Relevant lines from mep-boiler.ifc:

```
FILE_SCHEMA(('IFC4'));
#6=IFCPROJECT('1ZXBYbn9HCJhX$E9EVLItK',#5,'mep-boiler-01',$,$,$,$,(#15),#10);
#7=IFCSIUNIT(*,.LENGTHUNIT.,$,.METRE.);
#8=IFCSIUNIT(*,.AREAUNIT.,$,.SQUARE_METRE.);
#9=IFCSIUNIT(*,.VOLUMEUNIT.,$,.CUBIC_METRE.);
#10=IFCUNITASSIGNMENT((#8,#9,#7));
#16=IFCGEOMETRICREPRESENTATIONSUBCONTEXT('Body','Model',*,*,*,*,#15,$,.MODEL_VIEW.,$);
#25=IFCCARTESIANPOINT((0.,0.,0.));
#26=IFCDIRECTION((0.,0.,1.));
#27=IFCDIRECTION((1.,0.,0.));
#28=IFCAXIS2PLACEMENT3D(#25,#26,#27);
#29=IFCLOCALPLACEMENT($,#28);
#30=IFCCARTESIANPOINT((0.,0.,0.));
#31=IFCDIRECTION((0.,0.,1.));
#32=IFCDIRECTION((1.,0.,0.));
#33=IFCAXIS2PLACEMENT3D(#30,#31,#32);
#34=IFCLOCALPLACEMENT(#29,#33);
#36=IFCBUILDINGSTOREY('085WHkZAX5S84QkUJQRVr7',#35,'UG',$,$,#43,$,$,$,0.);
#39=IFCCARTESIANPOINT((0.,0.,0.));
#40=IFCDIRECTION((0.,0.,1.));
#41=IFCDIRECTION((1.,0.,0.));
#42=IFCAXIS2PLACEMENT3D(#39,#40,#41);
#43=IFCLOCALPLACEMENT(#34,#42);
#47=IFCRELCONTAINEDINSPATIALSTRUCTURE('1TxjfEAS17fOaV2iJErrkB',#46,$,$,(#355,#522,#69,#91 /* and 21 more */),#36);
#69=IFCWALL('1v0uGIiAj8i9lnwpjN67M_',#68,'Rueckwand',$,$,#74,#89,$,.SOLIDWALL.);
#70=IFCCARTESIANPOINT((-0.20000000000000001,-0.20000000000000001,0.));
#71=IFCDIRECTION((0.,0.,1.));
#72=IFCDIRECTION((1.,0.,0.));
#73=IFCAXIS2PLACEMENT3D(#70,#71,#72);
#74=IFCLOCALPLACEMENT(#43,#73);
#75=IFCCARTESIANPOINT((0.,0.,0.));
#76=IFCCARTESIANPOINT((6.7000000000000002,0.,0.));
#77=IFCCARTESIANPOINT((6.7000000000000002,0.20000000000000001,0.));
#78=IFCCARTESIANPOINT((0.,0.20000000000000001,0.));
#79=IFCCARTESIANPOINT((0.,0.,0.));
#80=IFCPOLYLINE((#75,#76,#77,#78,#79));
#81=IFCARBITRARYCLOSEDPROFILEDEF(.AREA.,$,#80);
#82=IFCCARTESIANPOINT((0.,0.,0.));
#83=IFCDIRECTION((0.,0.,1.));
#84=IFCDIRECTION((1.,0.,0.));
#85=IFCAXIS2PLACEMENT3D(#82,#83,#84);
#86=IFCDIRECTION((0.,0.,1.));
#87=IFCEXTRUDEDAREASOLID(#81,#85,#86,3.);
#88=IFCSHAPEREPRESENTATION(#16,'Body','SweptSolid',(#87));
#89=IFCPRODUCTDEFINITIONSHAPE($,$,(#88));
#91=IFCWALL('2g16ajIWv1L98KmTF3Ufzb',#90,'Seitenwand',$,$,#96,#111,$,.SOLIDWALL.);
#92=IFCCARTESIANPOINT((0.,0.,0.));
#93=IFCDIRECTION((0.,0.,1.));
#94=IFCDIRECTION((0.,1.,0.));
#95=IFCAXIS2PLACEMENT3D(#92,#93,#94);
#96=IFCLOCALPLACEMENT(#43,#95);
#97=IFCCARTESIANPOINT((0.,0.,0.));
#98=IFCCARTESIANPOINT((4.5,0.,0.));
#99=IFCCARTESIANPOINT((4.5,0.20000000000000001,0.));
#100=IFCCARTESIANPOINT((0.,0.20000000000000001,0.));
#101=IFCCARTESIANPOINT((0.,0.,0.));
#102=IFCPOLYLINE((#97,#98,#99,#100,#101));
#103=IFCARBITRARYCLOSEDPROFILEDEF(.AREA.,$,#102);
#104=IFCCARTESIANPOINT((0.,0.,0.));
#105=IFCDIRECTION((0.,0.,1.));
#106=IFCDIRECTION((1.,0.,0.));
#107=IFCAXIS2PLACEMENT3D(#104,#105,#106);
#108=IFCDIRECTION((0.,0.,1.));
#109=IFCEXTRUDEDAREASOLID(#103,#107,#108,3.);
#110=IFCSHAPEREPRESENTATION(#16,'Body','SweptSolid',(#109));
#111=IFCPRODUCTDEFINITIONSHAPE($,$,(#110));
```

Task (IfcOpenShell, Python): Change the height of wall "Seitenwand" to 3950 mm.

```python
import ifcopenshell
import ifcopenshell.geom
import ifcopenshell.util.representation
import ifcopenshell.util.shape

model = ifcopenshell.open("mep-boiler.ifc")
settings = ifcopenshell.geom.settings()


def volume(element):
    """Net volume in cubic metres, openings subtracted."""
    shape = ifcopenshell.geom.create_shape(settings, element)
    return ifcopenshell.util.shape.get_volume(shape.geometry)


wall = model.by_guid("2g16ajIWv1L98KmTF3Ufzb")
before = volume(wall)

body = ifcopenshell.util.representation.get_representation(wall, "Model", "Body")
solid = body.Items[0]
old_height = solid.Depth
solid.Depth = 3.95
after = volume(wall)

print(f"height {old_height:g} -> {solid.Depth:g}, volume {before:.3f} -> {after:.3f} m3")

model.write("mep-boiler_rev.ifc")
```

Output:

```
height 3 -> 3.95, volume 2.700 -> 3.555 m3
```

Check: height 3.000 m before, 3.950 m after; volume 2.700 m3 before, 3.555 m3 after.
